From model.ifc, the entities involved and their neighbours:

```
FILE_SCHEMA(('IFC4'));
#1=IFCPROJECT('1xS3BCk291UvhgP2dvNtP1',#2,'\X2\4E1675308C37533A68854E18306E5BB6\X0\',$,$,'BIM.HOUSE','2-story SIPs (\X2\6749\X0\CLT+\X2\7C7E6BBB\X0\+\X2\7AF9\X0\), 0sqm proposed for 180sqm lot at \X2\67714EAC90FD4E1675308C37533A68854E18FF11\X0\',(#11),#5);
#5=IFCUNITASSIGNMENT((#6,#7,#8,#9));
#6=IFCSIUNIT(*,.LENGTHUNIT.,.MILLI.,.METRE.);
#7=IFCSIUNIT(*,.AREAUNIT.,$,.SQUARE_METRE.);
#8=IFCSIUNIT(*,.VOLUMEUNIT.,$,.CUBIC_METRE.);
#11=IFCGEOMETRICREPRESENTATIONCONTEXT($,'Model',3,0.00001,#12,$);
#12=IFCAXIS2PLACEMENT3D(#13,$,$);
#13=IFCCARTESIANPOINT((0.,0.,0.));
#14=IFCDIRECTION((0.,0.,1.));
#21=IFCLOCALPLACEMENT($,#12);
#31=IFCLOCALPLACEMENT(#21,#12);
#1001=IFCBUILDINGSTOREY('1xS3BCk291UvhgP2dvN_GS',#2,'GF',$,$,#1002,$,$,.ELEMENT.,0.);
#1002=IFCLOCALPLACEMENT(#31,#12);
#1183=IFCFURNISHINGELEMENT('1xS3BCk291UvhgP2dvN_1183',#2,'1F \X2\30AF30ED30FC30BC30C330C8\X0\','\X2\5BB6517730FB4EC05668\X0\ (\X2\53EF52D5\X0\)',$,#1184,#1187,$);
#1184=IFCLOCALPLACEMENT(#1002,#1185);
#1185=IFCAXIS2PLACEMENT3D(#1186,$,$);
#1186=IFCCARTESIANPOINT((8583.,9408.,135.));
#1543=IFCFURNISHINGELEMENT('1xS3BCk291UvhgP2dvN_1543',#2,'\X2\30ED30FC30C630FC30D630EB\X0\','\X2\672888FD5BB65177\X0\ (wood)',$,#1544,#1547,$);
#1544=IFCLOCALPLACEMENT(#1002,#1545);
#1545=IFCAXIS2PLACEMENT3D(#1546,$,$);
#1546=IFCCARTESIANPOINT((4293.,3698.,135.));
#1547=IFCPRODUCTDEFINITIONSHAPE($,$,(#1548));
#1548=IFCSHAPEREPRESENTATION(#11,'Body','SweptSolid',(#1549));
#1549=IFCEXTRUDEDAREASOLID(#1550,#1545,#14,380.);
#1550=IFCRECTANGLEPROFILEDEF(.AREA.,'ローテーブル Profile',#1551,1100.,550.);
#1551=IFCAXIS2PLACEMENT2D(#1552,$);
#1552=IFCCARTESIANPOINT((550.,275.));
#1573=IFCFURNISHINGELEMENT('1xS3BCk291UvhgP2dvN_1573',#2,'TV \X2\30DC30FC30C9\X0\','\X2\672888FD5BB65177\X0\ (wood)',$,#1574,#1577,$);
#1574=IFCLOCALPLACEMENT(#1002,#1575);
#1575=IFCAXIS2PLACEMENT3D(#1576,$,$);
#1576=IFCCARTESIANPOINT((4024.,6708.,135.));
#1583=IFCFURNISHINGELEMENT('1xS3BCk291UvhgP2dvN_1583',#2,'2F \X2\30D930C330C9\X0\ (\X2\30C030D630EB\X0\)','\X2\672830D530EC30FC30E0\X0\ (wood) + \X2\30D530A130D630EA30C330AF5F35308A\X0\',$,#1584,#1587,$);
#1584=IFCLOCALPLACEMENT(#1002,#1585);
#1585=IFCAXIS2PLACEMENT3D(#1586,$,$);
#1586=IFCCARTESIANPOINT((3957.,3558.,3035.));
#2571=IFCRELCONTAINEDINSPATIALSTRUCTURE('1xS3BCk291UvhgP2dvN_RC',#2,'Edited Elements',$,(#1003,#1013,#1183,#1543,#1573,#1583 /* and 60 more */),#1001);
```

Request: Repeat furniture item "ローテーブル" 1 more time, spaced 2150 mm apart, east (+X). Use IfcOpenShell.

```python
import numpy as np
import ifcopenshell
import ifcopenshell.api.geometry
import ifcopenshell.api.root
import ifcopenshell.util.element
import ifcopenshell.util.placement

model = ifcopenshell.open("model.ifc")


def reuse_history(source, copy):
    """copy_class also copies each property set's owner history, people and application; keep the originals."""
    for rel in copy.IsDefinedBy:
        if rel.is_a("IfcRelDefinesByProperties") and (history := rel.RelatingPropertyDefinition.OwnerHistory):
            rel.RelatingPropertyDefinition.OwnerHistory = source.OwnerHistory
            ifcopenshell.util.element.remove_deep2(model, history)


source = model.by_guid("1xS3BCk291UvhgP2dvN_1543")
base = ifcopenshell.util.placement.get_local_placement(source.ObjectPlacement)
step = np.array([1.0, 0.0, 0.0]) * 2150.0

for i in range(1, 2):
    copy = ifcopenshell.api.root.copy_class(model, product=source)
    copy.Representation = ifcopenshell.util.element.copy_deep(
        model, source.Representation, exclude=["IfcGeometricRepresentationContext", "IfcRepresentationMap"]
    )
    reuse_history(source, copy)
    matrix = base.copy()
    matrix[:3, 3] += i * step
    print("added at", matrix[:3, 3].round(3) + 0.0)
    ifcopenshell.api.geometry.edit_object_placement(model, product=copy, matrix=matrix, is_si=False)

model.write("model-out.ifc")
```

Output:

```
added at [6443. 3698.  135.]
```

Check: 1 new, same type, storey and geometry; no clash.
